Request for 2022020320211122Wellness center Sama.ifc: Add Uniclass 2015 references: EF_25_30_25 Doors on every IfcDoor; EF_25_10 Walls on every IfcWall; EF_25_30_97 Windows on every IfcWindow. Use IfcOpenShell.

First a look at what the model holds.

```python
import ifcopenshell

model = ifcopenshell.open("2022020320211122Wellness center Sama.ifc")
print(model.schema)
print("classifications:", [c.Name for c in model.by_type("IfcClassification")])
for ifc_class in ("IfcDoor", "IfcRoof", "IfcStair", "IfcWall", "IfcWindow"):
    print(ifc_class, len(model.by_type(ifc_class)))
```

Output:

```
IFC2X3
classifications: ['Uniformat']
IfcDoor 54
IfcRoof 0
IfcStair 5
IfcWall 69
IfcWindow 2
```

```python
import ifcopenshell
import ifcopenshell.api.classification

model = ifcopenshell.open("2022020320211122Wellness center Sama.ifc")

# IFC2X3 requires Source and Edition and has no link from the project to the system.
system = model.create_entity("IfcClassification", Source="NBS", Edition="2015", Name="Uniclass 2015")

codes = {
    "IfcDoor": ("EF_25_30_25", "Doors"),
    "IfcWall": ("EF_25_10", "Walls"),
    "IfcWindow": ("EF_25_30_97", "Windows"),
}
for ifc_class, (code, name) in codes.items():
    products = model.by_type(ifc_class)
    ifcopenshell.api.classification.add_reference(
        model, products=products, classification=system, identification=code, name=name
    )
    print(code, len(products))

model.write("2022020320211122Wellness center Sama_v2.ifc")
```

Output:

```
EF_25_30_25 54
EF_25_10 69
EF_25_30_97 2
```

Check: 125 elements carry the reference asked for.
